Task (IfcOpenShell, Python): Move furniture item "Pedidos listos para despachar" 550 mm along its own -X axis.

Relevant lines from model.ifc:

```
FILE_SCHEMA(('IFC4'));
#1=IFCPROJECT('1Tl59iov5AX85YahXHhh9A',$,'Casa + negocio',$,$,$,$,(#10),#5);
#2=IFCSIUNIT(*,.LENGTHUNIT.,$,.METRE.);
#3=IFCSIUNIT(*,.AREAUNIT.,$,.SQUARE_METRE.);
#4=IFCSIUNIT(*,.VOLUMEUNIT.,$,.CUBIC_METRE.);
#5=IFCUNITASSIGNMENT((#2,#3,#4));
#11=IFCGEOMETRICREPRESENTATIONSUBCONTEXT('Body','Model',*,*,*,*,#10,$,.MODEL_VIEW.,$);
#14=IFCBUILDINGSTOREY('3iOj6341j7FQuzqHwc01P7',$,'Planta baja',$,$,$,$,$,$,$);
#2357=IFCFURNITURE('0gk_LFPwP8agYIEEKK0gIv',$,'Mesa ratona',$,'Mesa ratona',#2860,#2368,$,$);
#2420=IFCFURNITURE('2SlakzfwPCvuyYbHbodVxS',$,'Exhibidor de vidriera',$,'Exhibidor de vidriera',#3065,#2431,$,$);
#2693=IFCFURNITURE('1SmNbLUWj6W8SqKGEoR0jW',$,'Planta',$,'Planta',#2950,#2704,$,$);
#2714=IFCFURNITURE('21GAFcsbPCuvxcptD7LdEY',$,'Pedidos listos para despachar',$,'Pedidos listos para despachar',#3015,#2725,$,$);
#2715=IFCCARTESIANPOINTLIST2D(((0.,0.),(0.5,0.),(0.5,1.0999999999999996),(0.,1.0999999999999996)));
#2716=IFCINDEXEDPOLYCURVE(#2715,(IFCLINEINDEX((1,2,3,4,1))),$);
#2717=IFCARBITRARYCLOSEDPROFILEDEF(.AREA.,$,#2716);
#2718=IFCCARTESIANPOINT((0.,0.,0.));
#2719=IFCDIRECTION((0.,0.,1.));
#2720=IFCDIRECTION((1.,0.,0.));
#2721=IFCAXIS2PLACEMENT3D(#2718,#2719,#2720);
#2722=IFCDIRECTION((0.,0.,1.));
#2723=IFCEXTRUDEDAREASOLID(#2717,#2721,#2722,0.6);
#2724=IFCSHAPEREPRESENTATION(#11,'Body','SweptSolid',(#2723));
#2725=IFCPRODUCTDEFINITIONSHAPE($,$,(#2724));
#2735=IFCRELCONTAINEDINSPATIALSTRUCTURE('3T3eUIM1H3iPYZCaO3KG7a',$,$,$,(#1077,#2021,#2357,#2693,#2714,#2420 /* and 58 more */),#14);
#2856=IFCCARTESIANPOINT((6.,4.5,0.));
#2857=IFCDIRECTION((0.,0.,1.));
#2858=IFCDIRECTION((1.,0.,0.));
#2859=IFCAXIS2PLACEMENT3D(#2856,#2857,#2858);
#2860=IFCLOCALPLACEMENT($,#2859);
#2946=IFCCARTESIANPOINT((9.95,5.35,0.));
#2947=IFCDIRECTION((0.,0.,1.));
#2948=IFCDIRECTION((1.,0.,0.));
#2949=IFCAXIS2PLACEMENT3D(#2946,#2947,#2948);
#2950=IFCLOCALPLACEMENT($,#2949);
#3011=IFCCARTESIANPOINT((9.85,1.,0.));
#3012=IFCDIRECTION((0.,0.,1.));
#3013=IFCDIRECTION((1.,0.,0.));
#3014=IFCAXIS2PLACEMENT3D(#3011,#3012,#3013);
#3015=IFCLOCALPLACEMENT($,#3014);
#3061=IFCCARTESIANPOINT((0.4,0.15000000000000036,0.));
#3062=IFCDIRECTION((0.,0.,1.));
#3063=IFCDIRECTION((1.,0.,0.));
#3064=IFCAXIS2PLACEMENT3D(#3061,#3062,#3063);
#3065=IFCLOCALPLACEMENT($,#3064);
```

```python
import ifcopenshell
import ifcopenshell.api.geometry
import ifcopenshell.util.placement

model = ifcopenshell.open("model.ifc")

item = model.by_guid("21GAFcsbPCuvxcptD7LdEY")
matrix = ifcopenshell.util.placement.get_local_placement(item.ObjectPlacement)
matrix[:3, 3] -= matrix[:3, 0] * 0.55
ifcopenshell.api.geometry.edit_object_placement(model, product=item, matrix=matrix, is_si=False)

print(ifcopenshell.util.placement.get_local_placement(item.ObjectPlacement).round(3) + 0.0)

model.write("model_rev.ifc")
```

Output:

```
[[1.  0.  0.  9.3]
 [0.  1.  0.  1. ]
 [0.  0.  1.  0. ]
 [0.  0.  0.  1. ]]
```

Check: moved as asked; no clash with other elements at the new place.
